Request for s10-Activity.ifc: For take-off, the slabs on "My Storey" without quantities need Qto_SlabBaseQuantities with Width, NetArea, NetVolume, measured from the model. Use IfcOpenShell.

First a look at what the model holds.

```python
import ifcopenshell
import ifcopenshell.util.element
import ifcopenshell.util.unit

model = ifcopenshell.open("s10-Activity.ifc")
print(model.schema)
for unit_type in ("LENGTHUNIT", "AREAUNIT", "VOLUMEUNIT"):
    print(unit_type, ifcopenshell.util.unit.calculate_unit_scale(model, unit_type))
storey = next(s for s in model.by_type("IfcBuildingStorey") if s.Name == "My Storey")
slabs = [e for e in ifcopenshell.util.element.get_decomposition(storey) if e.is_a("IfcSlab")]
for e in sorted(slabs, key=lambda e: e.id()):
    print(e.id(), e.is_a(), e.Name, list(ifcopenshell.util.element.get_psets(e, qtos_only=True)), sep=" | ")
```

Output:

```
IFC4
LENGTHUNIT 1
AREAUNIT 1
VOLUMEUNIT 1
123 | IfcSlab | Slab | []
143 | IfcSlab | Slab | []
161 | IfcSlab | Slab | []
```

```python
import ifcopenshell
import ifcopenshell.api.pset
import ifcopenshell.geom
import ifcopenshell.util.element
import ifcopenshell.util.shape
import ifcopenshell.util.unit

model = ifcopenshell.open("s10-Activity.ifc")
unit_scale = ifcopenshell.util.unit.calculate_unit_scale(model)
area_scale = ifcopenshell.util.unit.calculate_unit_scale(model, "AREAUNIT")
volume_scale = ifcopenshell.util.unit.calculate_unit_scale(model, "VOLUMEUNIT")
settings = ifcopenshell.geom.settings()

storey = next(s for s in model.by_type("IfcBuildingStorey") if s.Name == "My Storey")
slabs = [e for e in ifcopenshell.util.element.get_decomposition(storey) if e.is_a("IfcSlab")]

for e in sorted(slabs, key=lambda e: e.id()):
    if ifcopenshell.util.element.get_psets(e, qtos_only=True, should_inherit=False):
        continue
    # Geometry comes back in metres, in the element's own axes.
    shape = ifcopenshell.geom.create_shape(settings, e)
    values = {
        "Width": ifcopenshell.util.shape.get_z(shape.geometry) / unit_scale,
        "NetArea": ifcopenshell.util.shape.get_footprint_area(shape.geometry) / area_scale,
        "NetVolume": ifcopenshell.util.shape.get_volume(shape.geometry) / volume_scale,
    }
    qto = ifcopenshell.api.pset.add_qto(model, product=e, name="Qto_SlabBaseQuantities")
    ifcopenshell.api.pset.edit_qto(model, qto=qto, properties=values)
    print(e.id(), {k: round(v, 3) for k, v in values.items()})

model.write("s10-Activity_v2.ifc")
```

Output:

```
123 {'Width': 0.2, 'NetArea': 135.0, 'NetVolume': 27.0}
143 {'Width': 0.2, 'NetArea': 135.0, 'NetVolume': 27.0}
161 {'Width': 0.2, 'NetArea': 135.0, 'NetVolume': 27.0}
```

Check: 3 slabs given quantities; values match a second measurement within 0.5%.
